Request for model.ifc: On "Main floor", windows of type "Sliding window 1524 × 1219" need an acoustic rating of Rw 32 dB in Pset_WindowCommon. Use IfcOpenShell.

First a look at what the model holds.

```python
import ifcopenshell
import ifcopenshell.util.element

model = ifcopenshell.open("model.ifc")
print(model.schema)
storey = next(s for s in model.by_type("IfcBuildingStorey") if s.Name == "Main floor")
windows = [e for e in ifcopenshell.util.element.get_decomposition(storey) if e.is_a("IfcWindow")]
seen = {}
for e in windows:
    element_type = ifcopenshell.util.element.get_type(e)
    key = (element_type.Name if element_type != e and element_type else None, ifcopenshell.util.element.get_pset(e, "Pset_WindowCommon", "AcousticRating"))
    seen[key] = seen.get(key, 0) + 1
for (name, value), count in sorted(seen.items(), key=str):
    print(count, "x", name, "|", value)
```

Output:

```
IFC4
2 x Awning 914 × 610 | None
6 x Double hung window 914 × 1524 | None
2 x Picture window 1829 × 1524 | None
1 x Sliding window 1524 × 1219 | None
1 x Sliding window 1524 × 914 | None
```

```python
import ifcopenshell
import ifcopenshell.api.pset
import ifcopenshell.util.element

model = ifcopenshell.open("model.ifc")

storey = next(s for s in model.by_type("IfcBuildingStorey") if s.Name == "Main floor")
windows = [e for e in ifcopenshell.util.element.get_decomposition(storey) if e.is_a("IfcWindow")]

count = 0
for e in windows:
    element_type = ifcopenshell.util.element.get_type(e)
    if element_type in (None, e) or element_type.Name != "Sliding window 1524 × 1219":
        continue
    # add_pset returns the element's existing set when there is one.
    pset = ifcopenshell.api.pset.add_pset(model, product=e, name="Pset_WindowCommon")
    ifcopenshell.api.pset.edit_pset(model, pset=pset, properties={"AcousticRating": "Rw 32 dB"})
    count += 1

print(count, "windows updated")

model.write("model-out.ifc")
```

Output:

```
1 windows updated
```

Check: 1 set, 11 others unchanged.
